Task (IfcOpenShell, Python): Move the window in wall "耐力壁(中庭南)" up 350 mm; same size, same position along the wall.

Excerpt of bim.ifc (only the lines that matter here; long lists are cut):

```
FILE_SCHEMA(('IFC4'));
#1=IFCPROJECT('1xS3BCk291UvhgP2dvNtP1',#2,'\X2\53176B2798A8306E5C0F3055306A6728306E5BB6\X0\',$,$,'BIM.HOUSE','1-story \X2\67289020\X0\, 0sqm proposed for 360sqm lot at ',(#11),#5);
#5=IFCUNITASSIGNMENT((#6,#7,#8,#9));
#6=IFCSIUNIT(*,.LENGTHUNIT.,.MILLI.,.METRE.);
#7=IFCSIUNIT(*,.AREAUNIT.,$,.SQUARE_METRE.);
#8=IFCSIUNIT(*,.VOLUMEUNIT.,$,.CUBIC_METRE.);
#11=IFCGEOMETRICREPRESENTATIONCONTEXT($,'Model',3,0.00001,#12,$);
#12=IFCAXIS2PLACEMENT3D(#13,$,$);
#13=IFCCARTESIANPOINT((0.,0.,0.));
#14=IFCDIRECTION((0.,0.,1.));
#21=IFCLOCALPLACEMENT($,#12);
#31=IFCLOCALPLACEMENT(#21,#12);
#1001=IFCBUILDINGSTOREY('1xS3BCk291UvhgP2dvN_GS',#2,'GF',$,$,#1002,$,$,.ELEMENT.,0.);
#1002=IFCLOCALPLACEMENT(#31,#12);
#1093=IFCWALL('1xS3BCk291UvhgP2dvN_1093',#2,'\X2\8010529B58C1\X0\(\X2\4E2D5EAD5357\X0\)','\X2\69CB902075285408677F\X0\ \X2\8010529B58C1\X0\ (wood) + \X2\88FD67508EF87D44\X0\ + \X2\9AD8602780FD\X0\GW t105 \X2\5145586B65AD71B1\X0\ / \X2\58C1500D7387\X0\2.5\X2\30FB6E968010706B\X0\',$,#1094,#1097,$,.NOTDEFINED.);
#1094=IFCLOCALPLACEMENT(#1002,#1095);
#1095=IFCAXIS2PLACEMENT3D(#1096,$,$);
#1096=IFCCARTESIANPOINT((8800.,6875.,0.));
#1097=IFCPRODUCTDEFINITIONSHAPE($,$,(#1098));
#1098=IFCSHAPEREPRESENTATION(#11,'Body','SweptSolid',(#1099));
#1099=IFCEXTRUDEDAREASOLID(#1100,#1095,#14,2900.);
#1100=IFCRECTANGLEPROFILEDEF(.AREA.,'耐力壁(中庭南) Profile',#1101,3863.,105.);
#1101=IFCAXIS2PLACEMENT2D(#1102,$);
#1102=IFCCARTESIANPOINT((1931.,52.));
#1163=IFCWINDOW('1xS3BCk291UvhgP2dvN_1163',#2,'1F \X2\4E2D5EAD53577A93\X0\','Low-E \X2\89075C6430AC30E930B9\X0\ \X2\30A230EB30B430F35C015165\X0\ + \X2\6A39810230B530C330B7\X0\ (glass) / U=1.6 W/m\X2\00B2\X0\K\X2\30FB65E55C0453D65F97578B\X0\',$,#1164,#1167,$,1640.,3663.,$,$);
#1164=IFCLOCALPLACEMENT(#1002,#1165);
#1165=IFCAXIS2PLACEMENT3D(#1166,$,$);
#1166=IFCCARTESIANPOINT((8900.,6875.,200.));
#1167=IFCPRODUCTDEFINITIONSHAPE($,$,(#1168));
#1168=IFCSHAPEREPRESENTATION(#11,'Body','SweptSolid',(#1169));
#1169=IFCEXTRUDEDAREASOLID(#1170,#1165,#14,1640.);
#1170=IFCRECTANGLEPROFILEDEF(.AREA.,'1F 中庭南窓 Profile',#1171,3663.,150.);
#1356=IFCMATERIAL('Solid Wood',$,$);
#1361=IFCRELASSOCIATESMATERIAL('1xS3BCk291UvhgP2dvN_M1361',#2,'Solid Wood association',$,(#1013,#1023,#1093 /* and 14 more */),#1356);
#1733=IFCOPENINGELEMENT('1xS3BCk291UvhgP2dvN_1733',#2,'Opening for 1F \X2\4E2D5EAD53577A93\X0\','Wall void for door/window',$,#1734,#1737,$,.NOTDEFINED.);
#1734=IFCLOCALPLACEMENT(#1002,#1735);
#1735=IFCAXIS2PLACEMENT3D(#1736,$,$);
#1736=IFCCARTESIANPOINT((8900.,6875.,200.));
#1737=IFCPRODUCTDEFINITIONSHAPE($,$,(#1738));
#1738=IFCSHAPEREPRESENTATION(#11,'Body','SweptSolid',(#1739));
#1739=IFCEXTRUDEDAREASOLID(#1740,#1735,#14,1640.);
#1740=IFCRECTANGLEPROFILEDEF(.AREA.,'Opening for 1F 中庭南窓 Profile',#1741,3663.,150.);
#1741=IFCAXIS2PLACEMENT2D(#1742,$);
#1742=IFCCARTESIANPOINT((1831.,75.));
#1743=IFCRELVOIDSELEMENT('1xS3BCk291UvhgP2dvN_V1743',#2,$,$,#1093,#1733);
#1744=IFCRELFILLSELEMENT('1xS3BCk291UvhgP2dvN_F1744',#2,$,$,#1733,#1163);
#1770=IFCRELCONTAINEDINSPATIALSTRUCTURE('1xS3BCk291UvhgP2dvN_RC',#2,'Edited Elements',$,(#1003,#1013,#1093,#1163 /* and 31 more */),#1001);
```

```python
import numpy as np
import ifcopenshell
import ifcopenshell.api.geometry
import ifcopenshell.util.placement
import ifcopenshell.util.unit

model = ifcopenshell.open("bim.ifc")
unit_scale = ifcopenshell.util.unit.calculate_unit_scale(model)

window = model.by_id(1163)
opening = window.FillsVoids[0].RelatingOpeningElement
dz = 350.0

shift = np.array([0.0, 0.0, dz])
# The window is not placed relative to its opening, so move both.
for product in (opening, window):
    matrix = ifcopenshell.util.placement.get_local_placement(product.ObjectPlacement)
    matrix[:3, 3] += shift
    ifcopenshell.api.geometry.edit_object_placement(model, product=product, matrix=matrix, is_si=False)

print(f"moved by {dz * unit_scale:+.3f} m")

model.write("bim_updated.ifc")
```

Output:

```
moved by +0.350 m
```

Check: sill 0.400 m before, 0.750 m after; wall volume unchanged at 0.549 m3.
